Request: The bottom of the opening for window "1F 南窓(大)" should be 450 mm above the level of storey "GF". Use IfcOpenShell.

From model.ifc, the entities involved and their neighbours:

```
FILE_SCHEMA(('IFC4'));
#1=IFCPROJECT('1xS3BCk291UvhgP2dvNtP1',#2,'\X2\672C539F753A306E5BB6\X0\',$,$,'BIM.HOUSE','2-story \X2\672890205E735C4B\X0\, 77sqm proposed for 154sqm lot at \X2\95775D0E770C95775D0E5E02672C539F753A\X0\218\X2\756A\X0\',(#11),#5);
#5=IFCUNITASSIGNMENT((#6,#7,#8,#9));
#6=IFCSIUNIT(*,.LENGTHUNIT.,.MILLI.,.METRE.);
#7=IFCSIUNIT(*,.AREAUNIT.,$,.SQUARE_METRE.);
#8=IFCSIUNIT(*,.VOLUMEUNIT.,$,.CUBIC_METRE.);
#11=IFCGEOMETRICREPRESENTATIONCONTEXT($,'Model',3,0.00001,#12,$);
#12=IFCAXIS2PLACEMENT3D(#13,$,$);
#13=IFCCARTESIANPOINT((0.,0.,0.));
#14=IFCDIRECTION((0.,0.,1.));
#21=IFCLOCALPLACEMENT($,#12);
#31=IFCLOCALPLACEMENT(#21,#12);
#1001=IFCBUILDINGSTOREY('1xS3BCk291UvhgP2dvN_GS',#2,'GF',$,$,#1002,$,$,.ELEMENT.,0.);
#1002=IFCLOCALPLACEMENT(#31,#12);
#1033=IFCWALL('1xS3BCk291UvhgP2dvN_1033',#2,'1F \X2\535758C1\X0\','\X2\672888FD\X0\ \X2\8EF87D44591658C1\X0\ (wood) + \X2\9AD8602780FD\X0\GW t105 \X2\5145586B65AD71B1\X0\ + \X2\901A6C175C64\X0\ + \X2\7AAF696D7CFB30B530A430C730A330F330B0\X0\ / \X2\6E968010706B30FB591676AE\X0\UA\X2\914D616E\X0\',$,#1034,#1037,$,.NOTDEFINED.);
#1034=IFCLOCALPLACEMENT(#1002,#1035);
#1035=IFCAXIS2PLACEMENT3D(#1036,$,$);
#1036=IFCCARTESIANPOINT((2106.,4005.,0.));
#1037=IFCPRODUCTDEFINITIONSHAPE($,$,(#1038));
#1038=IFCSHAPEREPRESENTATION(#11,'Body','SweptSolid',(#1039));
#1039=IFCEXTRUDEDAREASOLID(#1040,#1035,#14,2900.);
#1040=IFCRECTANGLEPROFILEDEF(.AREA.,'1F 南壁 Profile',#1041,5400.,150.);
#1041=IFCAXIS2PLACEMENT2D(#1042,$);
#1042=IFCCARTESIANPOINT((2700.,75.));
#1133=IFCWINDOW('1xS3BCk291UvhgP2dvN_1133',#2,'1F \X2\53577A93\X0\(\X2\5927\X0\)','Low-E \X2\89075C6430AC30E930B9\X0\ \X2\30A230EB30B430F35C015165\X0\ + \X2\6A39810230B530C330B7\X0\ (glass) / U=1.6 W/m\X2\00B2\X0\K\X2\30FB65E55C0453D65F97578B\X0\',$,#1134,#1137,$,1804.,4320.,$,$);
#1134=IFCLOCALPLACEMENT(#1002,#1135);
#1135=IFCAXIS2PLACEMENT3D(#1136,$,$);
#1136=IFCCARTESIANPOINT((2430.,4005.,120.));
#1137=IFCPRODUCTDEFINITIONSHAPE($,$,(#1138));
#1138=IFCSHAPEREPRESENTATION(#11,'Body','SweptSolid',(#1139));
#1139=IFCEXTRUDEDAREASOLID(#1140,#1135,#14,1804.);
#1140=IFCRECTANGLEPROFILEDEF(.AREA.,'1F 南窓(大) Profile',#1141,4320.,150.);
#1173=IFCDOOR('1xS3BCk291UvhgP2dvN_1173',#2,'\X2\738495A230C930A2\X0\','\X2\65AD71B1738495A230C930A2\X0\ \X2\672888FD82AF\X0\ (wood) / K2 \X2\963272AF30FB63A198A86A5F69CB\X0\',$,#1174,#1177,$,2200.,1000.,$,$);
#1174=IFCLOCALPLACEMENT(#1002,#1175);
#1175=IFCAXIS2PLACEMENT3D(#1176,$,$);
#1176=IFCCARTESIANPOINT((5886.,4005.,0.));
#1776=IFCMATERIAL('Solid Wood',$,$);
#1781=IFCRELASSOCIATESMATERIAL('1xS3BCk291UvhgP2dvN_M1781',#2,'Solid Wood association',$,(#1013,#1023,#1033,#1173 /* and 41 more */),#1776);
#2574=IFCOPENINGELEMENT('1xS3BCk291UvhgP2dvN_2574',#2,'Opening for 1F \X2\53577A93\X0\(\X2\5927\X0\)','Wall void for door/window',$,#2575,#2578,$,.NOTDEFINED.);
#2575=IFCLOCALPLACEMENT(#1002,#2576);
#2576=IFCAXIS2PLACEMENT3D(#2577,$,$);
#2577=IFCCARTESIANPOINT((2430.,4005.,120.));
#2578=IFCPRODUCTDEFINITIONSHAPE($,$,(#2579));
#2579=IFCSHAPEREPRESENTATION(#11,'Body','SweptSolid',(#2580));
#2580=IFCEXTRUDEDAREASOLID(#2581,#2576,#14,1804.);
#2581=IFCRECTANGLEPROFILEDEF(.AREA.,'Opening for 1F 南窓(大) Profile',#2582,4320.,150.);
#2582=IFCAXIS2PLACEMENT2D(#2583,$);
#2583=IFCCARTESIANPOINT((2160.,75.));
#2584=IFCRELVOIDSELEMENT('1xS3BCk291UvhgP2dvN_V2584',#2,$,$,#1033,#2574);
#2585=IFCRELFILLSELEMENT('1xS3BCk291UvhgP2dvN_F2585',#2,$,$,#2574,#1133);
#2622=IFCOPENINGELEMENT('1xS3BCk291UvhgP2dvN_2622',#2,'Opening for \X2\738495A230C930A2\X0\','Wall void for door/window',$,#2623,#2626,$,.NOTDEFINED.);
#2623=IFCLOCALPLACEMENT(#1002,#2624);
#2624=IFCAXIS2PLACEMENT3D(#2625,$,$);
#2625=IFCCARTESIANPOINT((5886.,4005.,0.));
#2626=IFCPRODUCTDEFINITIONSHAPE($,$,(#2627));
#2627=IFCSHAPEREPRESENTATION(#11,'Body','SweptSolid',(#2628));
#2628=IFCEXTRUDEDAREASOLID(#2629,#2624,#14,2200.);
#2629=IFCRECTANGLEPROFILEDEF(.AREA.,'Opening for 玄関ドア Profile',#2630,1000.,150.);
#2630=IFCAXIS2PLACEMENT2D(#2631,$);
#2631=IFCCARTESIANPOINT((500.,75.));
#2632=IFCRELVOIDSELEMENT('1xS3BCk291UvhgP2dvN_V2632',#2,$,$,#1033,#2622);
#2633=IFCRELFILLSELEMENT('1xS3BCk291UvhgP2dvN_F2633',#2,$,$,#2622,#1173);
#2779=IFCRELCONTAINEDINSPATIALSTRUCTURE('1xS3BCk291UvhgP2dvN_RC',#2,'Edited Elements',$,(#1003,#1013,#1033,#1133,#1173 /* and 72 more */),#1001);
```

```python
import numpy as np
import ifcopenshell
import ifcopenshell.api.geometry
import ifcopenshell.geom
import ifcopenshell.util.element
import ifcopenshell.util.placement
import ifcopenshell.util.shape
import ifcopenshell.util.unit

model = ifcopenshell.open("model.ifc")
unit_scale = ifcopenshell.util.unit.calculate_unit_scale(model)

window = model.by_guid("1xS3BCk291UvhgP2dvN_1133")
opening = window.FillsVoids[0].RelatingOpeningElement
storey = ifcopenshell.util.element.get_container(window, ifc_class="IfcBuildingStorey")
level = ifcopenshell.util.placement.get_local_placement(storey.ObjectPlacement)[2, 3]

# The opening's origin need not be at the sill, so measure its lowest point.
shape = ifcopenshell.geom.create_shape(ifcopenshell.geom.settings(), opening)
bottom = ifcopenshell.util.shape.get_shape_bottom_elevation(shape, shape.geometry) / unit_scale
dz = level + 0.45 / unit_scale - bottom

shift = np.array([0.0, 0.0, dz])
# The window is not placed relative to its opening, so move both.
for product in (opening, window):
    matrix = ifcopenshell.util.placement.get_local_placement(product.ObjectPlacement)
    matrix[:3, 3] += shift
    ifcopenshell.api.geometry.edit_object_placement(model, product=product, matrix=matrix, is_si=False)

print(f"moved by {dz * unit_scale:+.3f} m")

model.write("model_updated.ifc")
```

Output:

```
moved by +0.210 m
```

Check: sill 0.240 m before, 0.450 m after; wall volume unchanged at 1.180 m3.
